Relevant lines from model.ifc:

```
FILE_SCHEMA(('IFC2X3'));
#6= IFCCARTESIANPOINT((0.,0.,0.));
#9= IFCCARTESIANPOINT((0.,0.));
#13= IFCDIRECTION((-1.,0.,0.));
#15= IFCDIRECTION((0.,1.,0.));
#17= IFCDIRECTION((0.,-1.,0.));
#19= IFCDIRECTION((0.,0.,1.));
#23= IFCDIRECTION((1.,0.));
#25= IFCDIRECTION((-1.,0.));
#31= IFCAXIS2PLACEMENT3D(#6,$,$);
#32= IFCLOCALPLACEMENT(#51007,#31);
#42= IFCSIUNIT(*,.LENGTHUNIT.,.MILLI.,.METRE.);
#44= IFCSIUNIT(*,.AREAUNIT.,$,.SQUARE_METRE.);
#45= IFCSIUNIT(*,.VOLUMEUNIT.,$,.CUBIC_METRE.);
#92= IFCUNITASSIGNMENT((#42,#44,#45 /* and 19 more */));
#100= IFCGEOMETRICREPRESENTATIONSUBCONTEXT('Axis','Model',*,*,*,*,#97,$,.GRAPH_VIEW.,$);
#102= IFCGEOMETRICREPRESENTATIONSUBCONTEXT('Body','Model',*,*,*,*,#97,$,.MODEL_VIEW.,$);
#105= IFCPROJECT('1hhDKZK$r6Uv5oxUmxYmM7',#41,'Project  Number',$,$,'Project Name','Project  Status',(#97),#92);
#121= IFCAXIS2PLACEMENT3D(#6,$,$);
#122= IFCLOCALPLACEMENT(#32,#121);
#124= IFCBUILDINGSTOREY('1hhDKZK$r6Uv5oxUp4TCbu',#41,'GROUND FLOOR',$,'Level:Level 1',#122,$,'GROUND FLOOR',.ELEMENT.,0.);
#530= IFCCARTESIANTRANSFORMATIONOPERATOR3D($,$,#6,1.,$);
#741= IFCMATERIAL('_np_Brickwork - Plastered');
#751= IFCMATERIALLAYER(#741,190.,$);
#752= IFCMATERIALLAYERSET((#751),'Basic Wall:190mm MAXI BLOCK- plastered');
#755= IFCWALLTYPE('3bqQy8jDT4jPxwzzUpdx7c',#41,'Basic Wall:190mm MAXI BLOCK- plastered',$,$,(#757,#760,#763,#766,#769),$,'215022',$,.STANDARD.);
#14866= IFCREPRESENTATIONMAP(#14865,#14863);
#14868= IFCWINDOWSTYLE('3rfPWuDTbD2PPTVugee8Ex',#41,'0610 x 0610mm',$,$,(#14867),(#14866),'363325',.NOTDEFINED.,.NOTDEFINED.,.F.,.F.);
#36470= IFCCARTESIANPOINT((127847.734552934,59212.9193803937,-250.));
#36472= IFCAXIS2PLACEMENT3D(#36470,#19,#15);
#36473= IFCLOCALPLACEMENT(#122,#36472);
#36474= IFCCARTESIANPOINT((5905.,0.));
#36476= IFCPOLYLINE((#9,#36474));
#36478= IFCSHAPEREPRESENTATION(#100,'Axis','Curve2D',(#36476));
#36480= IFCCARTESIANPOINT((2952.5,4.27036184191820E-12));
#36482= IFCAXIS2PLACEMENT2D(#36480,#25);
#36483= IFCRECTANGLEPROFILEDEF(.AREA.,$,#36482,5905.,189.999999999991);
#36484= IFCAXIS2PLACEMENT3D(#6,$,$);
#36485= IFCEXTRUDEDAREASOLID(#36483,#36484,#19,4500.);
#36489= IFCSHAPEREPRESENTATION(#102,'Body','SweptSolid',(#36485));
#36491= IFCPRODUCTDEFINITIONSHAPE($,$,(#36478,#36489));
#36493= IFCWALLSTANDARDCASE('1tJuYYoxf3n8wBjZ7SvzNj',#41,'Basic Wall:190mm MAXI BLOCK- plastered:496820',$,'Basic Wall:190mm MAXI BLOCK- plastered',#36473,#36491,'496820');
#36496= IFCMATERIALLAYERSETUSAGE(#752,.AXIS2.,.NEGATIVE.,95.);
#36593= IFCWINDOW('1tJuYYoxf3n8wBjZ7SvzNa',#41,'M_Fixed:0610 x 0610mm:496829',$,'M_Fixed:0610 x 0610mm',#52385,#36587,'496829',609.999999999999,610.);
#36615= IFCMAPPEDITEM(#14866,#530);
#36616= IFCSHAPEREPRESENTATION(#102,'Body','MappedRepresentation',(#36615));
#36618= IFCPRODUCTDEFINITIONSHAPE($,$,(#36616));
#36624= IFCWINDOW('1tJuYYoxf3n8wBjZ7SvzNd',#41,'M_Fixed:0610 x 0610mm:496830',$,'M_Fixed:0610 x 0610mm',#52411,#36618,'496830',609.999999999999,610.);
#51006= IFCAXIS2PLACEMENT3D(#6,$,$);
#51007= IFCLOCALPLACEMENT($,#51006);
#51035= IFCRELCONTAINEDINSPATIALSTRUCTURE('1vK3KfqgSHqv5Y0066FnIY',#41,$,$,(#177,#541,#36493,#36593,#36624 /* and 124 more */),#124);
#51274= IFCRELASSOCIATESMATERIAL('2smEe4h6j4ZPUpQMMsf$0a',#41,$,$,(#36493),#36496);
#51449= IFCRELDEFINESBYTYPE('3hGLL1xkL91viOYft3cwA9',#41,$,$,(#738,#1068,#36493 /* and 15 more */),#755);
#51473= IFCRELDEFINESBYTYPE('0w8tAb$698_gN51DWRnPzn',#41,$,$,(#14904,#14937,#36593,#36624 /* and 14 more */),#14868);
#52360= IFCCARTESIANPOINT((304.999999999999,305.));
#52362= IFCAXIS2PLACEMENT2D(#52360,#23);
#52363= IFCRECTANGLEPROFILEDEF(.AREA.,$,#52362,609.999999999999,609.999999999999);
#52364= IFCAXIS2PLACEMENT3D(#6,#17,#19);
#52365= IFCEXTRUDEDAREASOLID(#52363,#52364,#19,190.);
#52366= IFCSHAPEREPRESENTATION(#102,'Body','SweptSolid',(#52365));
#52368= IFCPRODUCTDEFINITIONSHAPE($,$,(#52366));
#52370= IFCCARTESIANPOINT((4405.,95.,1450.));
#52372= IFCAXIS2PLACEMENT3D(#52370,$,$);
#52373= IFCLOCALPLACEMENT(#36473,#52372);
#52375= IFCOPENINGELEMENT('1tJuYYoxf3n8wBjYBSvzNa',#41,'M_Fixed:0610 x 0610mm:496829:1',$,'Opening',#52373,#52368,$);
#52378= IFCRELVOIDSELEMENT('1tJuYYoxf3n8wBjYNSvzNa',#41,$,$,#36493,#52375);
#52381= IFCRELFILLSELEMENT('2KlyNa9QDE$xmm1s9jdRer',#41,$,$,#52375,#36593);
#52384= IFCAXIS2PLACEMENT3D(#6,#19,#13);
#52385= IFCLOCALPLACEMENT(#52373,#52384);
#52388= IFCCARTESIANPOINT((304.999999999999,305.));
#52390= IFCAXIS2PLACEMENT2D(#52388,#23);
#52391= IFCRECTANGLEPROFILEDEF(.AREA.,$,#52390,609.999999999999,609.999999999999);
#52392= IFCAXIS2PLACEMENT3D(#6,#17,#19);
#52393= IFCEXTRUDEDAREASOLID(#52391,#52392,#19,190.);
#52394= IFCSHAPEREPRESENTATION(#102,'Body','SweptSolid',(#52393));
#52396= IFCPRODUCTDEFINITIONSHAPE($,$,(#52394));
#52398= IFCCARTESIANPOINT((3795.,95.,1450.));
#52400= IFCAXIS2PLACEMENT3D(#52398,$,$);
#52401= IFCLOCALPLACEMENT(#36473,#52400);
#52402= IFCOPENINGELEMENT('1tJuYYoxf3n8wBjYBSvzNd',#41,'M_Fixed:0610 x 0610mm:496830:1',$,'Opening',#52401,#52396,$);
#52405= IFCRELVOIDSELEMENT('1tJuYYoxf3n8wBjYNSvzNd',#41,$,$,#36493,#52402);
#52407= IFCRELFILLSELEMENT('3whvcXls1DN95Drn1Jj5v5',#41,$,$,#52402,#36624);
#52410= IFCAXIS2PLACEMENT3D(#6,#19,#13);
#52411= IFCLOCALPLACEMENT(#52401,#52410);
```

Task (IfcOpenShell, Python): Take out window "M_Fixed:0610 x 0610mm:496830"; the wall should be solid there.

```python
import ifcopenshell
import ifcopenshell.api.feature
import ifcopenshell.api.root
import ifcopenshell.geom
import ifcopenshell.util.shape

model = ifcopenshell.open("model.ifc")
settings = ifcopenshell.geom.settings()


def volume(element):
    """Net volume in cubic metres, openings subtracted."""
    shape = ifcopenshell.geom.create_shape(settings, element)
    return ifcopenshell.util.shape.get_volume(shape.geometry)


window = model.by_id(36624)
opening = window.FillsVoids[0].RelatingOpeningElement
wall = opening.VoidsElements[0].RelatingBuildingElement
before = volume(wall)

ifcopenshell.api.root.remove_product(model, product=window)
ifcopenshell.api.feature.remove_feature(model, feature=opening)

after = volume(wall)

print(f"wall volume {before:.3f} -> {after:.3f} m3")

model.write("model-out.ifc")
```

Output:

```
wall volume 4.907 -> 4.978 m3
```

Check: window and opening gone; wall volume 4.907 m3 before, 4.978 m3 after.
